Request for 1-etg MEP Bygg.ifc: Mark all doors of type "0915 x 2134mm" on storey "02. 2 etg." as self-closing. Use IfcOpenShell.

First a look at what the model holds.

```python
import ifcopenshell
import ifcopenshell.util.element

model = ifcopenshell.open("1-etg MEP Bygg.ifc")
print(model.schema)
storey = next(s for s in model.by_type("IfcBuildingStorey") if s.Name == "02. 2 etg.")
doors = [e for e in ifcopenshell.util.element.get_decomposition(storey) if e.is_a("IfcDoor")]
seen = {}
for e in doors:
    element_type = ifcopenshell.util.element.get_type(e)
    key = (element_type.Name if element_type != e and element_type else None, ifcopenshell.util.element.get_pset(e, "Pset_DoorCommon", "SelfClosing"))
    seen[key] = seen.get(key, 0) + 1
for (name, value), count in sorted(seen.items(), key=str):
    print(count, "x", name, "|", value)
```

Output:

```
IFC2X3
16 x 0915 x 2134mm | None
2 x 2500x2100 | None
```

```python
import ifcopenshell
import ifcopenshell.api.pset
import ifcopenshell.util.element

model = ifcopenshell.open("1-etg MEP Bygg.ifc")

storey = next(s for s in model.by_type("IfcBuildingStorey") if s.Name == "02. 2 etg.")
doors = [e for e in ifcopenshell.util.element.get_decomposition(storey) if e.is_a("IfcDoor")]

count = 0
for e in doors:
    element_type = ifcopenshell.util.element.get_type(e)
    if element_type in (None, e) or element_type.Name != "0915 x 2134mm":
        continue
    # add_pset returns the element's existing set when there is one.
    pset = ifcopenshell.api.pset.add_pset(model, product=e, name="Pset_DoorCommon")
    ifcopenshell.api.pset.edit_pset(model, pset=pset, properties={"SelfClosing": True})
    count += 1

print(count, "doors updated")

model.write("1-etg MEP Bygg_rev.ifc")
```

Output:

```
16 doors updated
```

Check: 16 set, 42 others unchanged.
